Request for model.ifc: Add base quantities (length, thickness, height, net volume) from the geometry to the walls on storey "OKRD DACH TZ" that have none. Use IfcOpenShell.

First a look at what the model holds.

```python
import ifcopenshell
import ifcopenshell.util.element
import ifcopenshell.util.unit

model = ifcopenshell.open("model.ifc")
print(model.schema)
for unit_type in ("LENGTHUNIT", "AREAUNIT", "VOLUMEUNIT"):
    print(unit_type, ifcopenshell.util.unit.calculate_unit_scale(model, unit_type))
storey = next(s for s in model.by_type("IfcBuildingStorey") if s.Name == "OKRD DACH TZ")
walls = [e for e in ifcopenshell.util.element.get_decomposition(storey) if e.is_a("IfcWall")]
for e in sorted(walls, key=lambda e: e.id()):
    print(e.id(), e.is_a(), e.Name, list(ifcopenshell.util.element.get_psets(e, qtos_only=True)), sep=" | ")
```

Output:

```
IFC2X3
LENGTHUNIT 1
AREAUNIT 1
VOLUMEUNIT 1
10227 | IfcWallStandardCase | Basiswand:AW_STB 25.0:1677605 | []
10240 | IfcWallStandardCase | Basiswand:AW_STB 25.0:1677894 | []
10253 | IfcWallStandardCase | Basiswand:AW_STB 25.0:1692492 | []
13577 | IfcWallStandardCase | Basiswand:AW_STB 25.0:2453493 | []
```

```python
import ifcopenshell
import ifcopenshell.api.pset
import ifcopenshell.geom
import ifcopenshell.util.element
import ifcopenshell.util.shape
import ifcopenshell.util.unit

model = ifcopenshell.open("model.ifc")
unit_scale = ifcopenshell.util.unit.calculate_unit_scale(model)
volume_scale = ifcopenshell.util.unit.calculate_unit_scale(model, "VOLUMEUNIT")
settings = ifcopenshell.geom.settings()

storey = next(s for s in model.by_type("IfcBuildingStorey") if s.Name == "OKRD DACH TZ")
walls = [e for e in ifcopenshell.util.element.get_decomposition(storey) if e.is_a("IfcWall")]

for e in sorted(walls, key=lambda e: e.id()):
    if ifcopenshell.util.element.get_psets(e, qtos_only=True, should_inherit=False):
        continue
    # Geometry comes back in metres, in the element's own axes.
    shape = ifcopenshell.geom.create_shape(settings, e)
    values = {
        "Length": ifcopenshell.util.shape.get_x(shape.geometry) / unit_scale,
        "Width": ifcopenshell.util.shape.get_y(shape.geometry) / unit_scale,
        "Height": ifcopenshell.util.shape.get_z(shape.geometry) / unit_scale,
        "NetVolume": ifcopenshell.util.shape.get_volume(shape.geometry) / volume_scale,
    }
    qto = ifcopenshell.api.pset.add_qto(model, product=e, name="BaseQuantities")
    ifcopenshell.api.pset.edit_qto(model, qto=qto, properties=values)
    print(e.id(), {k: round(v, 3) for k, v in values.items()})

model.write("model_edited.ifc")
```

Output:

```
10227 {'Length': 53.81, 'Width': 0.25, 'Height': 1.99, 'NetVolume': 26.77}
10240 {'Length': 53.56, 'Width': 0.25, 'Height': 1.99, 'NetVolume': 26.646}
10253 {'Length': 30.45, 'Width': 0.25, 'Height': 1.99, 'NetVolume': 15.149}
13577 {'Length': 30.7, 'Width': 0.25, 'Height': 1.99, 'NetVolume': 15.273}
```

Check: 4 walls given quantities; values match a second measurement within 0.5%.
